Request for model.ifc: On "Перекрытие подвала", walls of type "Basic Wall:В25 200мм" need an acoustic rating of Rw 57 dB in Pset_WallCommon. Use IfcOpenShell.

First a look at what the model holds.

```python
import ifcopenshell
import ifcopenshell.util.element

model = ifcopenshell.open("model.ifc")
print(model.schema)
storey = next(s for s in model.by_type("IfcBuildingStorey") if s.Name == "Перекрытие подвала")
walls = [e for e in ifcopenshell.util.element.get_decomposition(storey) if e.is_a("IfcWall")]
seen = {}
for e in walls:
    element_type = ifcopenshell.util.element.get_type(e)
    key = (element_type.Name if element_type != e and element_type else None, ifcopenshell.util.element.get_pset(e, "Pset_WallCommon", "AcousticRating"))
    seen[key] = seen.get(key, 0) + 1
for (name, value), count in sorted(seen.items(), key=str):
    print(count, "x", name, "|", value)
```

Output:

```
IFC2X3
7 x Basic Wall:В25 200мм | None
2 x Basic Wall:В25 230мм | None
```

```python
import ifcopenshell
import ifcopenshell.api.pset
import ifcopenshell.util.element

model = ifcopenshell.open("model.ifc")

storey = next(s for s in model.by_type("IfcBuildingStorey") if s.Name == "Перекрытие подвала")
walls = [e for e in ifcopenshell.util.element.get_decomposition(storey) if e.is_a("IfcWall")]

count = 0
for e in walls:
    element_type = ifcopenshell.util.element.get_type(e)
    if element_type in (None, e) or element_type.Name != "Basic Wall:В25 200мм":
        continue
    # add_pset returns the element's existing set when there is one.
    pset = ifcopenshell.api.pset.add_pset(model, product=e, name="Pset_WallCommon")
    ifcopenshell.api.pset.edit_pset(model, pset=pset, properties={"AcousticRating": "Rw 57 dB"})
    count += 1

print(count, "walls updated")

model.write("model_updated.ifc")
```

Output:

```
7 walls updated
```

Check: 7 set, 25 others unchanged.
